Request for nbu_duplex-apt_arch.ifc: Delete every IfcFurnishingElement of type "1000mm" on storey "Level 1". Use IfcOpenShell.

First a look at what the model holds.

```python
import ifcopenshell
import ifcopenshell.util.element

model = ifcopenshell.open("nbu_duplex-apt_arch.ifc")
print(model.schema)
storey = next(s for s in model.by_type("IfcBuildingStorey") if s.Name == "Level 1")
furniture = [e for e in ifcopenshell.util.element.get_decomposition(storey) if e.is_a("IfcFurnishingElement")]
seen = {}
for e in furniture:
    element_type = ifcopenshell.util.element.get_type(e)
    name = element_type.Name if element_type not in (None, e) else None
    seen[name] = seen.get(name, 0) + 1
for name, count in sorted(seen.items(), key=str):
    print(count, "x", name)
```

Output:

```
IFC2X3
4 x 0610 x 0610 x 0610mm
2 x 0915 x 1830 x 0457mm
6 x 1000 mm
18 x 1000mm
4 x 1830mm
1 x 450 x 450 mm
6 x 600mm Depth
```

```python
import ifcopenshell
import ifcopenshell.api.root
import ifcopenshell.util.element

model = ifcopenshell.open("nbu_duplex-apt_arch.ifc")

storey = next(s for s in model.by_type("IfcBuildingStorey") if s.Name == "Level 1")
furniture = [e for e in ifcopenshell.util.element.get_decomposition(storey) if e.is_a("IfcFurnishingElement")]
targets = [e for e in furniture if (t := ifcopenshell.util.element.get_type(e)) not in (None, e) and t.Name == "1000mm"]

for e in targets:
    ifcopenshell.api.root.remove_product(model, product=e)
print(len(targets), "removed")

model.write("nbu_duplex-apt_arch_updated.ifc")
```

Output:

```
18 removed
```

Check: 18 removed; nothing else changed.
